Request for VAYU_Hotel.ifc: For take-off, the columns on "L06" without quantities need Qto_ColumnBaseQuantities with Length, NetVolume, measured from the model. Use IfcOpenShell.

First a look at what the model holds.

```python
import ifcopenshell
import ifcopenshell.util.element
import ifcopenshell.util.unit

model = ifcopenshell.open("VAYU_Hotel.ifc")
print(model.schema)
for unit_type in ("LENGTHUNIT", "AREAUNIT", "VOLUMEUNIT"):
    print(unit_type, ifcopenshell.util.unit.calculate_unit_scale(model, unit_type))
storey = next(s for s in model.by_type("IfcBuildingStorey") if s.Name == "L06")
columns = [e for e in ifcopenshell.util.element.get_decomposition(storey) if e.is_a("IfcColumn")]
for e in sorted(columns, key=lambda e: e.id()):
    print(e.id(), e.is_a(), e.Name, list(ifcopenshell.util.element.get_psets(e, qtos_only=True)), sep=" | ")
```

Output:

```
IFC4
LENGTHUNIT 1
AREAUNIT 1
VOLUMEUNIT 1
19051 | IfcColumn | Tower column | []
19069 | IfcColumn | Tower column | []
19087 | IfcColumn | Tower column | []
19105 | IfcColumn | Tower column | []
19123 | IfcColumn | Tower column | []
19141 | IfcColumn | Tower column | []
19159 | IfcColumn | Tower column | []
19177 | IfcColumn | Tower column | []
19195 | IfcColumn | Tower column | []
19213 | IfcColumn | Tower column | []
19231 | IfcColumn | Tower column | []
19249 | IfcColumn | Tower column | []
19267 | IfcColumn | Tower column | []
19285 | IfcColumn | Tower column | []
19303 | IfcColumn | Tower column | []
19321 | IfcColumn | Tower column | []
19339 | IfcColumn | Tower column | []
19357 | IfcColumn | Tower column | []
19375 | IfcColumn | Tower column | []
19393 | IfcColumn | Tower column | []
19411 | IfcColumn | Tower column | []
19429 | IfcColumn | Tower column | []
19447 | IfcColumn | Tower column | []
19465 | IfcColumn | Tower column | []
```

```python
import ifcopenshell
import ifcopenshell.api.pset
import ifcopenshell.geom
import ifcopenshell.util.element
import ifcopenshell.util.shape
import ifcopenshell.util.unit

model = ifcopenshell.open("VAYU_Hotel.ifc")
unit_scale = ifcopenshell.util.unit.calculate_unit_scale(model)
volume_scale = ifcopenshell.util.unit.calculate_unit_scale(model, "VOLUMEUNIT")
settings = ifcopenshell.geom.settings()

storey = next(s for s in model.by_type("IfcBuildingStorey") if s.Name == "L06")
columns = [e for e in ifcopenshell.util.element.get_decomposition(storey) if e.is_a("IfcColumn")]

for e in sorted(columns, key=lambda e: e.id()):
    if ifcopenshell.util.element.get_psets(e, qtos_only=True, should_inherit=False):
        continue
    # Geometry comes back in metres, in the element's own axes.
    shape = ifcopenshell.geom.create_shape(settings, e)
    values = {
        "Length": ifcopenshell.util.shape.get_z(shape.geometry) / unit_scale,
        "NetVolume": ifcopenshell.util.shape.get_volume(shape.geometry) / volume_scale,
    }
    qto = ifcopenshell.api.pset.add_qto(model, product=e, name="Qto_ColumnBaseQuantities")
    ifcopenshell.api.pset.edit_qto(model, qto=qto, properties=values)
    print(e.id(), {k: round(v, 3) for k, v in values.items()})

model.write("VAYU_Hotel_v2.ifc")
```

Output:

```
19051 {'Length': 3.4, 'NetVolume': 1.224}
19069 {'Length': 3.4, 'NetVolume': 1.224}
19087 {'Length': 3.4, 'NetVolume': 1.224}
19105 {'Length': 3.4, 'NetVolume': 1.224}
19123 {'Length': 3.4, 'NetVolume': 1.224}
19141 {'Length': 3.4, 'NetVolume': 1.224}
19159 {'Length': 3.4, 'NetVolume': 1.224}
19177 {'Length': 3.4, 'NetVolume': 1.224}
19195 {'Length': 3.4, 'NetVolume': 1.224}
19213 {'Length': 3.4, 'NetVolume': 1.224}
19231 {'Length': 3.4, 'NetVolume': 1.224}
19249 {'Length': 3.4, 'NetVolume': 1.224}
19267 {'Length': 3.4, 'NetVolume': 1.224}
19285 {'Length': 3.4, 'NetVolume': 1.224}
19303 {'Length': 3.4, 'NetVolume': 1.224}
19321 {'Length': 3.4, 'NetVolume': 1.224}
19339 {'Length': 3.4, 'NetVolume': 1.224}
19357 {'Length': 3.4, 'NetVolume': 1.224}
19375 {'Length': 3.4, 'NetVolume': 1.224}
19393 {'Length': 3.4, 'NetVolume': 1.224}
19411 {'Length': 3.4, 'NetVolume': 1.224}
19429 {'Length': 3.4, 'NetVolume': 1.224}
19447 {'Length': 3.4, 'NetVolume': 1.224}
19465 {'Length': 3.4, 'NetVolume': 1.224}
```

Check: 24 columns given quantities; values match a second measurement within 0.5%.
